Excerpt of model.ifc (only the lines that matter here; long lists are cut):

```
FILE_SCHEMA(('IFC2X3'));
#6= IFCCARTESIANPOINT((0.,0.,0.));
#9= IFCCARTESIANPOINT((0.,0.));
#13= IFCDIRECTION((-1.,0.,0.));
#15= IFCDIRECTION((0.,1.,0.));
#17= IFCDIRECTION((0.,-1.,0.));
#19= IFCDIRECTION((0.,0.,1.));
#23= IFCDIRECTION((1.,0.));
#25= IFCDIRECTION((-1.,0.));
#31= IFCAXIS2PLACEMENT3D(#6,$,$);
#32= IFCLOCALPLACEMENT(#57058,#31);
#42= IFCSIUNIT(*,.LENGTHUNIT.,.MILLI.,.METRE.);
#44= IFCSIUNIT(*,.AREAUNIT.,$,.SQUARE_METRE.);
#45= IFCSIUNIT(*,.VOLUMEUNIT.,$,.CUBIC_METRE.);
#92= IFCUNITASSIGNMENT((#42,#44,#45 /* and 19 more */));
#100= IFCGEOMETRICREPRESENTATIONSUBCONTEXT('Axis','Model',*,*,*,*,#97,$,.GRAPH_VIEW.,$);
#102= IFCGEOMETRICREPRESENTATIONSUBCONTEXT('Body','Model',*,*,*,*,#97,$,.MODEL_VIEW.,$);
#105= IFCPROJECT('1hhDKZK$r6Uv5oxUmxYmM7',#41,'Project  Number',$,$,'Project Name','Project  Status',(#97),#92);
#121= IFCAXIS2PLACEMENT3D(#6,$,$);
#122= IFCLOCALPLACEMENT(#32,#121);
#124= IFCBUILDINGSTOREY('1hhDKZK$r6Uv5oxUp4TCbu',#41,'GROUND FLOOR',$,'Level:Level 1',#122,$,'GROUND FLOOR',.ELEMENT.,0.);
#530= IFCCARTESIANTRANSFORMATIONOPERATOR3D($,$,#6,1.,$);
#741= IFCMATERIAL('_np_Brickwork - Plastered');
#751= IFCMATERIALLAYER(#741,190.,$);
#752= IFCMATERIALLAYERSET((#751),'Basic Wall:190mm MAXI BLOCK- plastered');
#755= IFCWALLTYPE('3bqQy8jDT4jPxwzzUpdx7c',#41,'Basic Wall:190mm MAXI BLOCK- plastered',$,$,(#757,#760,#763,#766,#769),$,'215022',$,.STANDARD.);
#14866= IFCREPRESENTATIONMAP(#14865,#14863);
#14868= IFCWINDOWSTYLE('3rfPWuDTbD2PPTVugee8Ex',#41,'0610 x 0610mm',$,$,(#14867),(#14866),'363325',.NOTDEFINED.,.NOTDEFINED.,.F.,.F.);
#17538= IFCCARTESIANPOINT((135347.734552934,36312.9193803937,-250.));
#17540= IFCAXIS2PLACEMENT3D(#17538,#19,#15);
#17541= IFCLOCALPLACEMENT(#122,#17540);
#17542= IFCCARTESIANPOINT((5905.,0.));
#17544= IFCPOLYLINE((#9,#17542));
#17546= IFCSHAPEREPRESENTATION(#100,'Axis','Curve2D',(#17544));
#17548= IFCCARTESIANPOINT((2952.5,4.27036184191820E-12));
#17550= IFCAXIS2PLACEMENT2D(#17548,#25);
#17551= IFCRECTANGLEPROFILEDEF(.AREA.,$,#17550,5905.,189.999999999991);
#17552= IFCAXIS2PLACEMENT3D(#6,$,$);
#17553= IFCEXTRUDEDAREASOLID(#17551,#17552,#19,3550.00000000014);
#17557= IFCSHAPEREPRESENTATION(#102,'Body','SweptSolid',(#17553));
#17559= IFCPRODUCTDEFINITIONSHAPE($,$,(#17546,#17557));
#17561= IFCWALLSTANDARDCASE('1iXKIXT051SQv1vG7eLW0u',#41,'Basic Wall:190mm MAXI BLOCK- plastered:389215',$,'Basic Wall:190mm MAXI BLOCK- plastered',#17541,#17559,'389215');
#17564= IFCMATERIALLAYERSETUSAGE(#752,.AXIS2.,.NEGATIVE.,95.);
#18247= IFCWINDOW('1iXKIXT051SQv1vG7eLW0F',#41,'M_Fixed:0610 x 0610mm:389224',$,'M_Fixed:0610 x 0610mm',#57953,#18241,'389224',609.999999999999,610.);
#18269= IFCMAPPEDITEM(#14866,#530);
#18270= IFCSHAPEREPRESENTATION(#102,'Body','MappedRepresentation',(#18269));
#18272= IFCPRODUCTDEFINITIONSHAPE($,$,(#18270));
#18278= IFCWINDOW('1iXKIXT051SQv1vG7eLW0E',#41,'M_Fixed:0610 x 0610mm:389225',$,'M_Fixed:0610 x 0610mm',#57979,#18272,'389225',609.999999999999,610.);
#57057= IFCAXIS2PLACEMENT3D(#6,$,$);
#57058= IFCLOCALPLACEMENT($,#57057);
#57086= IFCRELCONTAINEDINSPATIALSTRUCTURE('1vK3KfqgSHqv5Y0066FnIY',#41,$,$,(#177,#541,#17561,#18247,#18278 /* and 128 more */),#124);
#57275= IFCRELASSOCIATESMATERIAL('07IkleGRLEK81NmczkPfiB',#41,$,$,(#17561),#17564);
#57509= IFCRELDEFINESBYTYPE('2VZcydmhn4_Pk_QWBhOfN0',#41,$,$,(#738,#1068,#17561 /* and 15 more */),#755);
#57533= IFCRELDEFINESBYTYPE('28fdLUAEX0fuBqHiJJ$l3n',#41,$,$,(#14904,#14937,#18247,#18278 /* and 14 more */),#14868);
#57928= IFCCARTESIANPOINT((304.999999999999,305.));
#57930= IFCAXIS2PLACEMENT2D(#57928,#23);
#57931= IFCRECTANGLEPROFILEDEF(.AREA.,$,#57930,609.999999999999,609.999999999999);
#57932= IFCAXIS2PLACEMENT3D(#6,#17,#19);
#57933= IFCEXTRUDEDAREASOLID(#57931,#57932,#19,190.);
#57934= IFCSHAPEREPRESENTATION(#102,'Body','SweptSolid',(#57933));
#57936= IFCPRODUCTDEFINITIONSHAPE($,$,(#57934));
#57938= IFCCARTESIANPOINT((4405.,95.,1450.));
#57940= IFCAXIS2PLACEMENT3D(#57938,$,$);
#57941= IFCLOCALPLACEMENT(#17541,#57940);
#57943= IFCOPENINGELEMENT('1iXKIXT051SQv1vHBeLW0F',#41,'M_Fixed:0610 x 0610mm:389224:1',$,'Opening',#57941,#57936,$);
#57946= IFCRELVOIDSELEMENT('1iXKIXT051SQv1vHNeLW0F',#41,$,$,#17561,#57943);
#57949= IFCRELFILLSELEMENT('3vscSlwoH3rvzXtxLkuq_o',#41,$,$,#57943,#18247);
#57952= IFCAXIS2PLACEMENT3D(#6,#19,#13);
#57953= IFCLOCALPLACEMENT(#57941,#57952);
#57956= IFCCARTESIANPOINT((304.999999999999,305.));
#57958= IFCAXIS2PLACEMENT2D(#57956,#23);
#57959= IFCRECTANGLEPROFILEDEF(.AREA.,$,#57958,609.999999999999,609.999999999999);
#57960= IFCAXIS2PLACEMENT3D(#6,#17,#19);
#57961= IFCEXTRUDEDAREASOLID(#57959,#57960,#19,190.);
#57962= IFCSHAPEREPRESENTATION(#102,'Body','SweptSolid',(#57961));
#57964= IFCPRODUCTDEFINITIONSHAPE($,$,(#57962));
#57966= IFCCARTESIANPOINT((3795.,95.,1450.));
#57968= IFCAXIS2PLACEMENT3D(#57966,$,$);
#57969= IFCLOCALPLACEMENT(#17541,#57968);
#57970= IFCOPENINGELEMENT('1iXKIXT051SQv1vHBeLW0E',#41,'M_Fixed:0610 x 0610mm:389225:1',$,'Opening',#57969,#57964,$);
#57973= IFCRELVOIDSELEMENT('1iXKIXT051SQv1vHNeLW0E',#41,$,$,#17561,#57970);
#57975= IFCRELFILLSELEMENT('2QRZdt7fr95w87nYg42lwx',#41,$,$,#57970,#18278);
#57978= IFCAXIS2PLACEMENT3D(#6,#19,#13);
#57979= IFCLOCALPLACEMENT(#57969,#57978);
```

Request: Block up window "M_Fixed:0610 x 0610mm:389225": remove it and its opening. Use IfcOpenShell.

```python
import ifcopenshell
import ifcopenshell.api.feature
import ifcopenshell.api.root
import ifcopenshell.geom
import ifcopenshell.util.shape

model = ifcopenshell.open("model.ifc")
settings = ifcopenshell.geom.settings()


def volume(element):
    """Net volume in cubic metres, openings subtracted."""
    shape = ifcopenshell.geom.create_shape(settings, element)
    return ifcopenshell.util.shape.get_volume(shape.geometry)


window = model.by_guid("1iXKIXT051SQv1vG7eLW0E")
opening = window.FillsVoids[0].RelatingOpeningElement
wall = opening.VoidsElements[0].RelatingBuildingElement
before = volume(wall)

ifcopenshell.api.root.remove_product(model, product=window)
ifcopenshell.api.feature.remove_feature(model, feature=opening)

after = volume(wall)

print(f"wall volume {before:.3f} -> {after:.3f} m3")

model.write("model_edited.ifc")
```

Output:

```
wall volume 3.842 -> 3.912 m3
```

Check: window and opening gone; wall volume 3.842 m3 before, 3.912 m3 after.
